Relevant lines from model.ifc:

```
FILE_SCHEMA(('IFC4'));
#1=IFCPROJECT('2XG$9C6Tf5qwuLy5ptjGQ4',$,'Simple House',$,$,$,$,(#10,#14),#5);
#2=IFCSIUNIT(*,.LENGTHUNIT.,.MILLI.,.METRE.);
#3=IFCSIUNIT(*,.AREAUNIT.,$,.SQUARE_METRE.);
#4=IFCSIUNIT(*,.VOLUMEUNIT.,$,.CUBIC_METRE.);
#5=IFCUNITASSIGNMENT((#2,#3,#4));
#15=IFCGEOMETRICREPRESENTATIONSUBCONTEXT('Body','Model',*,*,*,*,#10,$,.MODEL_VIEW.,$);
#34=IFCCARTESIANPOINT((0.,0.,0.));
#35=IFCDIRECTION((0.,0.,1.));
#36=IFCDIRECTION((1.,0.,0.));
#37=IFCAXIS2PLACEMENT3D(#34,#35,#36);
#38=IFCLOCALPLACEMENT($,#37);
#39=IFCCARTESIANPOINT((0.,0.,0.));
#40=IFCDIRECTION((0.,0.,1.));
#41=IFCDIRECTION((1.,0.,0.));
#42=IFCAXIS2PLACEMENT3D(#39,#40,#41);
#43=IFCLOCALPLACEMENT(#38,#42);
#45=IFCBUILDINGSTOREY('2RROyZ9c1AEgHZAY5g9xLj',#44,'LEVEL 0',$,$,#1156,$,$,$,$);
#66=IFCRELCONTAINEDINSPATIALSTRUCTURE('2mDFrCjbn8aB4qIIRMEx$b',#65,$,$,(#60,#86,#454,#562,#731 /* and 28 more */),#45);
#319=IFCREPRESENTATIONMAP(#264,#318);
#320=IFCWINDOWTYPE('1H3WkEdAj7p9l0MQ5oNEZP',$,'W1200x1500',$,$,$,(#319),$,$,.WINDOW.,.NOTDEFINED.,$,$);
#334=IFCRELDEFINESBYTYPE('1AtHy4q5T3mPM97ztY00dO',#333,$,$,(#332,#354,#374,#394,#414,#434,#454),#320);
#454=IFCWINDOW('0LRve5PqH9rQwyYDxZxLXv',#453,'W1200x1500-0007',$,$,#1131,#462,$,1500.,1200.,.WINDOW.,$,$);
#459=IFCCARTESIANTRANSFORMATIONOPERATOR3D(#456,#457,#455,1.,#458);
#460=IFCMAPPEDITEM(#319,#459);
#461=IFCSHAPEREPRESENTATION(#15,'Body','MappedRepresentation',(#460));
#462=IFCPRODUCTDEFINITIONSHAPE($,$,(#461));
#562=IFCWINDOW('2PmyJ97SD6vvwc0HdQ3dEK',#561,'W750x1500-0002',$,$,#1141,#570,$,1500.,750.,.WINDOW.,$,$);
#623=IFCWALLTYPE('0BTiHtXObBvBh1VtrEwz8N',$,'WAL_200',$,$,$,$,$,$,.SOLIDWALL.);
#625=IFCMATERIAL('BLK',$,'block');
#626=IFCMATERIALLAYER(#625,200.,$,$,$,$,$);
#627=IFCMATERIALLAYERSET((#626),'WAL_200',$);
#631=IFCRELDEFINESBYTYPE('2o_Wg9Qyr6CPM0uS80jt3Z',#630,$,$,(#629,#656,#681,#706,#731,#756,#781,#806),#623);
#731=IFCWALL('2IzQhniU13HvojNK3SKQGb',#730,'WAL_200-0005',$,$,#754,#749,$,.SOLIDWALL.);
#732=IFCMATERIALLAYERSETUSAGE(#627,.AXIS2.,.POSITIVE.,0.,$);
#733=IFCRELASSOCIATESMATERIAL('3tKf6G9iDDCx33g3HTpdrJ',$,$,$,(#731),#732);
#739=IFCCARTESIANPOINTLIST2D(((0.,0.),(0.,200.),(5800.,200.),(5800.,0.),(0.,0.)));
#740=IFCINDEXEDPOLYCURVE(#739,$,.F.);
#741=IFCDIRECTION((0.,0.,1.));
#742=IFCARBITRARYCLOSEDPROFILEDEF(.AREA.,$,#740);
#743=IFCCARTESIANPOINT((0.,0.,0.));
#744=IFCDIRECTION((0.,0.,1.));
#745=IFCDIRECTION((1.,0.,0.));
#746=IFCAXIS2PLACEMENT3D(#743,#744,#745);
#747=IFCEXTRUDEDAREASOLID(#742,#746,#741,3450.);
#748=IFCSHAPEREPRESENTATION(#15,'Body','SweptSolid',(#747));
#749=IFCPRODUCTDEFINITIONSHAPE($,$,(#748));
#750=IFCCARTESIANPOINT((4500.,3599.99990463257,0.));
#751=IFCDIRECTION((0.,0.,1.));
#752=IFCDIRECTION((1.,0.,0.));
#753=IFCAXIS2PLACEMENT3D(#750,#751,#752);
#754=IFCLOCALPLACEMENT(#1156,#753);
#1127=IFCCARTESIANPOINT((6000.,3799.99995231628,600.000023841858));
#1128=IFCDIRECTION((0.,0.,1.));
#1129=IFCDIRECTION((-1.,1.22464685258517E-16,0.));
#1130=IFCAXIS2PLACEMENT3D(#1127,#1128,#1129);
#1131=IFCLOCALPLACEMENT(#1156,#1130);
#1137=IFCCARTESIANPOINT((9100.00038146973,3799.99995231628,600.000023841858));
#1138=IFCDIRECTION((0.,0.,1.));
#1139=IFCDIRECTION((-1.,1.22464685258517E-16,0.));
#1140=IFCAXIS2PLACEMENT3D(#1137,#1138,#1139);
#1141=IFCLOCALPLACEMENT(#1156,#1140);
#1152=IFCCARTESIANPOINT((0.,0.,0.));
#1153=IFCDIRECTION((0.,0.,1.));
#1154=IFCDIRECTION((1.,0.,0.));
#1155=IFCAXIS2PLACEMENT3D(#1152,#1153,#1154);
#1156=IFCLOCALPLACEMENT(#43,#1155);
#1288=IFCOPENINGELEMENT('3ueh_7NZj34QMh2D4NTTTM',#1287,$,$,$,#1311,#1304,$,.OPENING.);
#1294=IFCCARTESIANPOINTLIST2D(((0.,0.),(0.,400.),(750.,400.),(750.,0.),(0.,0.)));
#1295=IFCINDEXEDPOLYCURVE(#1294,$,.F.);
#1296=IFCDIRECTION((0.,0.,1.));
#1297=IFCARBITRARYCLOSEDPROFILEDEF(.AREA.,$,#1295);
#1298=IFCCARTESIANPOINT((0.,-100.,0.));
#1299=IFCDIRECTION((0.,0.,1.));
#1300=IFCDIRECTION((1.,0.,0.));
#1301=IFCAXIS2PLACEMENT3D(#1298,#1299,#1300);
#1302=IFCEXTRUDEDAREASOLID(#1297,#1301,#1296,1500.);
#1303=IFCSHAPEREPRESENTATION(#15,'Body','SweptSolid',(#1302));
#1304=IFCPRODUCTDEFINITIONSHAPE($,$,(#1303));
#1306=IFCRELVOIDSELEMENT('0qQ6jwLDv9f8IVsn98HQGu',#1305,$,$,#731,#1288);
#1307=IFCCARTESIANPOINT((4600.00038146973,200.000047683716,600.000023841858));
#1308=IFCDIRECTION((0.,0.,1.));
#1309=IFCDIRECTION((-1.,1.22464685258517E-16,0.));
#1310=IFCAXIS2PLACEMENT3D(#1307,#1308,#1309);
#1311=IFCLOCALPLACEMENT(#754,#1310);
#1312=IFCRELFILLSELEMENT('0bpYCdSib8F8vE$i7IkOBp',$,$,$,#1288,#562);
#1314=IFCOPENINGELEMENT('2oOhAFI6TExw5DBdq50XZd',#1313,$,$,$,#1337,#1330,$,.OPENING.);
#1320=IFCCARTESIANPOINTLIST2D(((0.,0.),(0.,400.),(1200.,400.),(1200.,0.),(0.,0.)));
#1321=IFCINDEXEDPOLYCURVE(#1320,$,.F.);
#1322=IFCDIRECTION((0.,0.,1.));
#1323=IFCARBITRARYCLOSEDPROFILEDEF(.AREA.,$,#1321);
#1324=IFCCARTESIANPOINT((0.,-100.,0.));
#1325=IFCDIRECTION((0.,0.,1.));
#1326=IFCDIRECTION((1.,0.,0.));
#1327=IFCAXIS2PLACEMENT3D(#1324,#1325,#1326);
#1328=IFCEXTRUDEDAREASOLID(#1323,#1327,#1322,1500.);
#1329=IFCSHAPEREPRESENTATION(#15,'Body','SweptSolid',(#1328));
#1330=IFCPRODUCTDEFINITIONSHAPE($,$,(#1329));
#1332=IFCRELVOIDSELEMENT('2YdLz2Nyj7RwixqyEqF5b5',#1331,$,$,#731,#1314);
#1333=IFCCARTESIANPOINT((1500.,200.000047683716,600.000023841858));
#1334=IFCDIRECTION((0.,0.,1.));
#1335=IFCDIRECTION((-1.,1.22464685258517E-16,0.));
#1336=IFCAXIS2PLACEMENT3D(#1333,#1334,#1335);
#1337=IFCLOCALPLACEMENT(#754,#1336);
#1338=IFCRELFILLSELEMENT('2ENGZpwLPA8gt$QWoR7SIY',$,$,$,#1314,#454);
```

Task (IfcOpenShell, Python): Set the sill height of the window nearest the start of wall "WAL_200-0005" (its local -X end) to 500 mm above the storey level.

```python
import numpy as np
import ifcopenshell
import ifcopenshell.api.geometry
import ifcopenshell.geom
import ifcopenshell.util.element
import ifcopenshell.util.placement
import ifcopenshell.util.shape
import ifcopenshell.util.unit

model = ifcopenshell.open("model.ifc")
unit_scale = ifcopenshell.util.unit.calculate_unit_scale(model)

window = model.by_guid("0LRve5PqH9rQwyYDxZxLXv")
opening = window.FillsVoids[0].RelatingOpeningElement
storey = ifcopenshell.util.element.get_container(window, ifc_class="IfcBuildingStorey")
level = ifcopenshell.util.placement.get_local_placement(storey.ObjectPlacement)[2, 3]

# The opening's origin need not be at the sill, so measure its lowest point.
shape = ifcopenshell.geom.create_shape(ifcopenshell.geom.settings(), opening)
bottom = ifcopenshell.util.shape.get_shape_bottom_elevation(shape, shape.geometry) / unit_scale
dz = level + 0.5 / unit_scale - bottom

shift = np.array([0.0, 0.0, dz])
# The window is not placed relative to its opening, so move both.
for product in (opening, window):
    matrix = ifcopenshell.util.placement.get_local_placement(product.ObjectPlacement)
    matrix[:3, 3] += shift
    ifcopenshell.api.geometry.edit_object_placement(model, product=product, matrix=matrix, is_si=False)

print(f"moved by {dz * unit_scale:+.3f} m")

model.write("model-out.ifc")
```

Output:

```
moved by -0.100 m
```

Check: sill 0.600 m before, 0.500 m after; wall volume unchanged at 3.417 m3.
